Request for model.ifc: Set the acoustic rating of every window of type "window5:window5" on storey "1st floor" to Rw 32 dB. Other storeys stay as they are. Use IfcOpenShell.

First a look at what the model holds.

```python
import ifcopenshell
import ifcopenshell.util.element

model = ifcopenshell.open("model.ifc")
print(model.schema)
storey = next(s for s in model.by_type("IfcBuildingStorey") if s.Name == "1st floor")
windows = [e for e in ifcopenshell.util.element.get_decomposition(storey) if e.is_a("IfcWindow")]
seen = {}
for e in windows:
    element_type = ifcopenshell.util.element.get_type(e)
    key = (element_type.Name if element_type != e and element_type else None, ifcopenshell.util.element.get_pset(e, "Pset_WindowCommon", "AcousticRating"))
    seen[key] = seen.get(key, 0) + 1
for (name, value), count in sorted(seen.items(), key=str):
    print(count, "x", name, "|", value)
```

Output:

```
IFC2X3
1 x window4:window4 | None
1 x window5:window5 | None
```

```python
import ifcopenshell
import ifcopenshell.api.pset
import ifcopenshell.util.element

model = ifcopenshell.open("model.ifc")

storey = next(s for s in model.by_type("IfcBuildingStorey") if s.Name == "1st floor")
windows = [e for e in ifcopenshell.util.element.get_decomposition(storey) if e.is_a("IfcWindow")]

count = 0
for e in windows:
    element_type = ifcopenshell.util.element.get_type(e)
    if element_type in (None, e) or element_type.Name != "window5:window5":
        continue
    # add_pset returns the element's existing set when there is one.
    pset = ifcopenshell.api.pset.add_pset(model, product=e, name="Pset_WindowCommon")
    ifcopenshell.api.pset.edit_pset(model, pset=pset, properties={"AcousticRating": "Rw 32 dB"})
    count += 1

print(count, "windows updated")

model.write("model_rev.ifc")
```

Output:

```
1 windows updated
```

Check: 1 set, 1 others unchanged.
